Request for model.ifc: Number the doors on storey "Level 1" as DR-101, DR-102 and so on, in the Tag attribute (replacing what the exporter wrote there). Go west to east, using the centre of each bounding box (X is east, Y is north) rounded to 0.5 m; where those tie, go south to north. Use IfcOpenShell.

First a look at what the model holds.

```python
import ifcopenshell
import ifcopenshell.util.element
import ifcopenshell.util.placement

model = ifcopenshell.open("model.ifc")
print(model.schema)
storey = next(s for s in model.by_type("IfcBuildingStorey") if s.Name == "Level 1")
doors = [e for e in ifcopenshell.util.element.get_decomposition(storey) if e.is_a("IfcDoor")]
for e in sorted(doors, key=lambda e: e.id()):
    origin = ifcopenshell.util.placement.get_local_placement(e.ObjectPlacement)[:3, 3]
    print(e.id(), e.Tag, e.Name, origin.round(2) + 0.0, sep=" | ")
```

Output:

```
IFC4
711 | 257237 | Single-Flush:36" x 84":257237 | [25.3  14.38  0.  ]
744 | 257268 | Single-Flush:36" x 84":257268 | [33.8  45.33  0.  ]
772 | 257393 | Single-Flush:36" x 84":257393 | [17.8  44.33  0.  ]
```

```python
import ifcopenshell
import ifcopenshell.geom
import ifcopenshell.util.element
import ifcopenshell.util.shape

model = ifcopenshell.open("model.ifc")
settings = ifcopenshell.geom.settings()
settings.set("use-world-coords", True)


def centre(element):
    shape = ifcopenshell.geom.create_shape(settings, element)
    return ifcopenshell.util.shape.get_bbox_centroid(shape.geometry)


storey = next(s for s in model.by_type("IfcBuildingStorey") if s.Name == "Level 1")
doors = [e for e in ifcopenshell.util.element.get_decomposition(storey) if e.is_a("IfcDoor")]

# Insertion points can sit at a corner or the storey origin, so sort by the geometry (in metres).
centres = {e: centre(e) for e in doors}
doors.sort(key=lambda e: (round(centres[e][0] / 0.5), centres[e][1]))

for i, e in enumerate(doors, start=1):
    number = f"DR-1{i:02d}"
    e.Tag = number
    print(e.id(), number)

model.write("model_edited.ifc")
```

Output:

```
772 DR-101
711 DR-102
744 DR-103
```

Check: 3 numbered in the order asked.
